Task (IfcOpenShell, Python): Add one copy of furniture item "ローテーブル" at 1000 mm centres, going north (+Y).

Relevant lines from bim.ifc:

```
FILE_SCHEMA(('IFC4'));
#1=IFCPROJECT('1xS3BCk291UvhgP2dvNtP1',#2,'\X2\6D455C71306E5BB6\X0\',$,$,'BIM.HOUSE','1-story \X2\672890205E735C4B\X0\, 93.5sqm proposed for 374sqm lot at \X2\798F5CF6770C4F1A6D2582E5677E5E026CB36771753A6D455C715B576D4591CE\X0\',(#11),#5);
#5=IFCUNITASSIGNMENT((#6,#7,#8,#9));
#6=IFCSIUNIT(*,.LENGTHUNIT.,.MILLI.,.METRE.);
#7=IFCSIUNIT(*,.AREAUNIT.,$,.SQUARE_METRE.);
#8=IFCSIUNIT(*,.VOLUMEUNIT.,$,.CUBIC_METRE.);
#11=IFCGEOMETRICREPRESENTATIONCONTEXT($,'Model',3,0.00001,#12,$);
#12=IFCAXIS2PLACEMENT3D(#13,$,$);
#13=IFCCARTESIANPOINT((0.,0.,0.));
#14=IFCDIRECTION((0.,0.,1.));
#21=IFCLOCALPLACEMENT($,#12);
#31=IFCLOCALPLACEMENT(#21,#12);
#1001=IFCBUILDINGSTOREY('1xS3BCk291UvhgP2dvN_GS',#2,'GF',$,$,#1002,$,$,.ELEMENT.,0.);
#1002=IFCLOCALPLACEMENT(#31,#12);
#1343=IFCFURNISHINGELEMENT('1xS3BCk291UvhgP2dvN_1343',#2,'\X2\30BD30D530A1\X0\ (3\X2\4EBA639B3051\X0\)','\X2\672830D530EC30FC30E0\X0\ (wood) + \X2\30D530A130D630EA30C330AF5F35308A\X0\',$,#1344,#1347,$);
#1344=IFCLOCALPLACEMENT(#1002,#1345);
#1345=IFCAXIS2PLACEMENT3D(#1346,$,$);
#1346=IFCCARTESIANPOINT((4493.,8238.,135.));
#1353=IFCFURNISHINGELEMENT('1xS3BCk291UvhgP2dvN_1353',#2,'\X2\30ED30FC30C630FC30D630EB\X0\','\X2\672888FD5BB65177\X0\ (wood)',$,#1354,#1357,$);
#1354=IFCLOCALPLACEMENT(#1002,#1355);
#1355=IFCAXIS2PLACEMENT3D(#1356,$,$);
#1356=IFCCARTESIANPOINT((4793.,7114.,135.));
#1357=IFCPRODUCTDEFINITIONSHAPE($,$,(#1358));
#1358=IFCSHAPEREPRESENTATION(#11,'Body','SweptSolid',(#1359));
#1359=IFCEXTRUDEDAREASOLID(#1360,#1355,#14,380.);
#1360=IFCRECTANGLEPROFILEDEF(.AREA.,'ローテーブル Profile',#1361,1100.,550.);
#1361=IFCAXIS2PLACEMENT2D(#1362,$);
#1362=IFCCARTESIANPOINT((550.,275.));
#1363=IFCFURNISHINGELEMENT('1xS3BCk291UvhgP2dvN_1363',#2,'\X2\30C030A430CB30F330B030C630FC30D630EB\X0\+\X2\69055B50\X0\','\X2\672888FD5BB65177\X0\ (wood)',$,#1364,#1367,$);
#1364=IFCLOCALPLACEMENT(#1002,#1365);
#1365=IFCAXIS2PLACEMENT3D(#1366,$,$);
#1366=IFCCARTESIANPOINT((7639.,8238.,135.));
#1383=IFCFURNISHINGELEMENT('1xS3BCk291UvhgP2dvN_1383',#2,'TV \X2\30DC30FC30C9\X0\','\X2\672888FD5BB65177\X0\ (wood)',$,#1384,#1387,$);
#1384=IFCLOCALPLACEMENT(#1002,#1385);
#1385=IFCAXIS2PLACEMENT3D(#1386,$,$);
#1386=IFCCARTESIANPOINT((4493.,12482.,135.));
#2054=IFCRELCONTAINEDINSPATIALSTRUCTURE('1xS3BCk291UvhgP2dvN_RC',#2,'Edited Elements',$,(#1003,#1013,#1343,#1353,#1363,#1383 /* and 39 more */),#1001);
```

```python
import numpy as np
import ifcopenshell
import ifcopenshell.api.geometry
import ifcopenshell.api.root
import ifcopenshell.util.element
import ifcopenshell.util.placement
import ifcopenshell.util.unit

model = ifcopenshell.open("bim.ifc")
unit_scale = ifcopenshell.util.unit.calculate_unit_scale(model)


def reuse_history(source, copy):
    """copy_class also copies each property set's owner history, people and application; keep the originals."""
    for rel in copy.IsDefinedBy:
        if rel.is_a("IfcRelDefinesByProperties") and (history := rel.RelatingPropertyDefinition.OwnerHistory):
            rel.RelatingPropertyDefinition.OwnerHistory = source.OwnerHistory
            ifcopenshell.util.element.remove_deep2(model, history)


source = model.by_guid("1xS3BCk291UvhgP2dvN_1353")
base = ifcopenshell.util.placement.get_local_placement(source.ObjectPlacement)
step = np.array([0.0, 1.0, 0.0]) * 1 / unit_scale

for i in range(1, 2):
    copy = ifcopenshell.api.root.copy_class(model, product=source)
    copy.Representation = ifcopenshell.util.element.copy_deep(
        model, source.Representation, exclude=["IfcGeometricRepresentationContext", "IfcRepresentationMap"]
    )
    reuse_history(source, copy)
    matrix = base.copy()
    matrix[:3, 3] += i * step
    print("added at", matrix[:3, 3].round(3) + 0.0)
    ifcopenshell.api.geometry.edit_object_placement(model, product=copy, matrix=matrix, is_si=False)

model.write("bim_rev.ifc")
```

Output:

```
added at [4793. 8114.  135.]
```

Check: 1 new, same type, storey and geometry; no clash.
